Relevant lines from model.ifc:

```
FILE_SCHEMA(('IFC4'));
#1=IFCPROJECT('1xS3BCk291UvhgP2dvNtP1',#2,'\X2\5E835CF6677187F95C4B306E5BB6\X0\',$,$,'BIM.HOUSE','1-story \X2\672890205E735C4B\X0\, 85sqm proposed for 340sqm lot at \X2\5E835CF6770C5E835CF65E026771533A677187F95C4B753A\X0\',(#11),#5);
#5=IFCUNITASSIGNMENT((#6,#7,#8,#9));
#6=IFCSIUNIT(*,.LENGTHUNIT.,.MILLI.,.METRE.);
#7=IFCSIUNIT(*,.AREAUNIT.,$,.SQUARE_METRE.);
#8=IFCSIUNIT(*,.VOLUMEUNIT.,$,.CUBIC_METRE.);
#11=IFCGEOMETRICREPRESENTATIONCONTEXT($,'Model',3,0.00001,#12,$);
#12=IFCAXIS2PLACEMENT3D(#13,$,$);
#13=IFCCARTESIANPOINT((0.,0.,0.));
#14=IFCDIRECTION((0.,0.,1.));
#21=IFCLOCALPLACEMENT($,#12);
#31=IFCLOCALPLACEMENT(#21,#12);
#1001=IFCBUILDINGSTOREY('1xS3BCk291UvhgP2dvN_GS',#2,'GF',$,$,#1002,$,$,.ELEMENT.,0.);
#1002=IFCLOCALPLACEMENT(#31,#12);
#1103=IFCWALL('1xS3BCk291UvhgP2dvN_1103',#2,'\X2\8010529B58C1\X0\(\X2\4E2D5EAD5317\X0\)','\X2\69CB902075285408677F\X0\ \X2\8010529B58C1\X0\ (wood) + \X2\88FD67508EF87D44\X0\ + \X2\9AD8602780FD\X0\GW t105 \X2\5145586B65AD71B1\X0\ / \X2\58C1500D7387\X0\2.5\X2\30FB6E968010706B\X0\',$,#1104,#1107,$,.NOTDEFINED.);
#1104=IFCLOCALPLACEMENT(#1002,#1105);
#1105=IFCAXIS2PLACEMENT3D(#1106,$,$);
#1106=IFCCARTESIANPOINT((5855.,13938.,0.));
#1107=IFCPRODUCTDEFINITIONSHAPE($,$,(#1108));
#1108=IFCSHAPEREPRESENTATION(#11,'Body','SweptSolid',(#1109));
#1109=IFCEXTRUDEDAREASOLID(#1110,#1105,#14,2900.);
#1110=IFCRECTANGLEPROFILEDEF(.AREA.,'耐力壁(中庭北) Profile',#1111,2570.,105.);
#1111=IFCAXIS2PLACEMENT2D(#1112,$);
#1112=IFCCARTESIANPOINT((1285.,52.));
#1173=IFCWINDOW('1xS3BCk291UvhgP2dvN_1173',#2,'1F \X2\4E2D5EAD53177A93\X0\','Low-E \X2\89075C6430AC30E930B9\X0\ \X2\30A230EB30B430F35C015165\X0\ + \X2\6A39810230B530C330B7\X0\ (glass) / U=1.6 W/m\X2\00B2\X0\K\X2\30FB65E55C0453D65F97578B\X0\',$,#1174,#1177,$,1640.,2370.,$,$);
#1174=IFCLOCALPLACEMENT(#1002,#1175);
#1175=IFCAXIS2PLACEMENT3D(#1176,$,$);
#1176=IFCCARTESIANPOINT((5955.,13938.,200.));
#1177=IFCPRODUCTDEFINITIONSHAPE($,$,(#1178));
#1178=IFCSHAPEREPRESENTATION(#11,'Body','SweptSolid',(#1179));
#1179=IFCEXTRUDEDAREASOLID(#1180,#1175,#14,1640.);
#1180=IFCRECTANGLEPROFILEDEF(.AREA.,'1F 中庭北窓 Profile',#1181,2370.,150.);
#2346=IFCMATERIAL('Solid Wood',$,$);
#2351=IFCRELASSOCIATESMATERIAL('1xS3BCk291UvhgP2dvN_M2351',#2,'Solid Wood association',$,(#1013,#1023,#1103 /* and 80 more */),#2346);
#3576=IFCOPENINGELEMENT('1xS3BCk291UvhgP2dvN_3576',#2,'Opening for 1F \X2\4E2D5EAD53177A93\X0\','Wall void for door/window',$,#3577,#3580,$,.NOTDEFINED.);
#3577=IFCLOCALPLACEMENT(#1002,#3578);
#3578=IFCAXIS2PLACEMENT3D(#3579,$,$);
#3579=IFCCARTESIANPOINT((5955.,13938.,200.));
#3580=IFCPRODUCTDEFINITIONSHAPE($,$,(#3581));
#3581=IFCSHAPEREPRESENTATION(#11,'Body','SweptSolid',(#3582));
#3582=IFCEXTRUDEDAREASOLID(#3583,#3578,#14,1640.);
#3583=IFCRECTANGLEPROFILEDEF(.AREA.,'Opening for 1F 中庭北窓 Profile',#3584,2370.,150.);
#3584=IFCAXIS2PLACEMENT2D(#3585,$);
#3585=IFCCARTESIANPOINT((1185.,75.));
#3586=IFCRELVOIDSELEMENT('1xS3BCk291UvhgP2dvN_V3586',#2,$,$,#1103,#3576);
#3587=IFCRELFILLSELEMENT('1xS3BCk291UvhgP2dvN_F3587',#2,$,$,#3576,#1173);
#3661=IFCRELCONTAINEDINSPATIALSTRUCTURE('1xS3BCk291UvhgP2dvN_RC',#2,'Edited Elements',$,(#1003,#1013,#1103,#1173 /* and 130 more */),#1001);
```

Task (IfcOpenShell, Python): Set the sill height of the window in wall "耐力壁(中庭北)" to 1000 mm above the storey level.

```python
import numpy as np
import ifcopenshell
import ifcopenshell.api.geometry
import ifcopenshell.geom
import ifcopenshell.util.element
import ifcopenshell.util.placement
import ifcopenshell.util.shape
import ifcopenshell.util.unit

model = ifcopenshell.open("model.ifc")
unit_scale = ifcopenshell.util.unit.calculate_unit_scale(model)

window = model.by_id(1173)
opening = window.FillsVoids[0].RelatingOpeningElement
storey = ifcopenshell.util.element.get_container(window, ifc_class="IfcBuildingStorey")
level = ifcopenshell.util.placement.get_local_placement(storey.ObjectPlacement)[2, 3]

# The opening's origin need not be at the sill, so measure its lowest point.
shape = ifcopenshell.geom.create_shape(ifcopenshell.geom.settings(), opening)
bottom = ifcopenshell.util.shape.get_shape_bottom_elevation(shape, shape.geometry) / unit_scale
dz = level + 1 / unit_scale - bottom

shift = np.array([0.0, 0.0, dz])
# The window is not placed relative to its opening, so move both.
for product in (opening, window):
    matrix = ifcopenshell.util.placement.get_local_placement(product.ObjectPlacement)
    matrix[:3, 3] += shift
    ifcopenshell.api.geometry.edit_object_placement(model, product=product, matrix=matrix, is_si=False)

print(f"moved by {dz * unit_scale:+.3f} m")

model.write("model-out.ifc")
```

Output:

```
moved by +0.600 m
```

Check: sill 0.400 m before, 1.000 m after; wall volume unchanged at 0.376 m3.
